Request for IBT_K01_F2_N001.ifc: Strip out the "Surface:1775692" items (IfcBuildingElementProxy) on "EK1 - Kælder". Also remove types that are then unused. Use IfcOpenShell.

First a look at what the model holds.

```python
import ifcopenshell
import ifcopenshell.util.element

model = ifcopenshell.open("IBT_K01_F2_N001.ifc")
print(model.schema)
storey = next(s for s in model.by_type("IfcBuildingStorey") if s.Name == "EK1 - Kælder")
proxies = [e for e in ifcopenshell.util.element.get_decomposition(storey) if e.is_a("IfcBuildingElementProxy")]
seen = {}
for e in proxies:
    element_type = ifcopenshell.util.element.get_type(e)
    name = element_type.Name if element_type not in (None, e) else None
    seen[name] = seen.get(name, 0) + 1
for name, count in sorted(seen.items(), key=str):
    print(count, "x", name)
```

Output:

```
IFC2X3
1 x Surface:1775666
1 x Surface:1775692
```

```python
import ifcopenshell
import ifcopenshell.api.root
import ifcopenshell.util.element

model = ifcopenshell.open("IBT_K01_F2_N001.ifc")

storey = next(s for s in model.by_type("IfcBuildingStorey") if s.Name == "EK1 - Kælder")
proxies = [e for e in ifcopenshell.util.element.get_decomposition(storey) if e.is_a("IfcBuildingElementProxy")]
targets = [e for e in proxies if (t := ifcopenshell.util.element.get_type(e)) not in (None, e) and t.Name == "Surface:1775692"]
types = {ifcopenshell.util.element.get_type(e) for e in targets} - {None, *targets}

for e in targets:
    ifcopenshell.api.root.remove_product(model, product=e)
print(len(targets), "removed")

unused = [t for t in types if not ifcopenshell.util.element.get_types(t)]
for t in unused:
    ifcopenshell.api.root.remove_product(model, product=t)
print(len(unused), "unused types removed")

model.write("IBT_K01_F2_N001_v2.ifc")
```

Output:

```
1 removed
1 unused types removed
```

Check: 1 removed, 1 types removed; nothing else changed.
